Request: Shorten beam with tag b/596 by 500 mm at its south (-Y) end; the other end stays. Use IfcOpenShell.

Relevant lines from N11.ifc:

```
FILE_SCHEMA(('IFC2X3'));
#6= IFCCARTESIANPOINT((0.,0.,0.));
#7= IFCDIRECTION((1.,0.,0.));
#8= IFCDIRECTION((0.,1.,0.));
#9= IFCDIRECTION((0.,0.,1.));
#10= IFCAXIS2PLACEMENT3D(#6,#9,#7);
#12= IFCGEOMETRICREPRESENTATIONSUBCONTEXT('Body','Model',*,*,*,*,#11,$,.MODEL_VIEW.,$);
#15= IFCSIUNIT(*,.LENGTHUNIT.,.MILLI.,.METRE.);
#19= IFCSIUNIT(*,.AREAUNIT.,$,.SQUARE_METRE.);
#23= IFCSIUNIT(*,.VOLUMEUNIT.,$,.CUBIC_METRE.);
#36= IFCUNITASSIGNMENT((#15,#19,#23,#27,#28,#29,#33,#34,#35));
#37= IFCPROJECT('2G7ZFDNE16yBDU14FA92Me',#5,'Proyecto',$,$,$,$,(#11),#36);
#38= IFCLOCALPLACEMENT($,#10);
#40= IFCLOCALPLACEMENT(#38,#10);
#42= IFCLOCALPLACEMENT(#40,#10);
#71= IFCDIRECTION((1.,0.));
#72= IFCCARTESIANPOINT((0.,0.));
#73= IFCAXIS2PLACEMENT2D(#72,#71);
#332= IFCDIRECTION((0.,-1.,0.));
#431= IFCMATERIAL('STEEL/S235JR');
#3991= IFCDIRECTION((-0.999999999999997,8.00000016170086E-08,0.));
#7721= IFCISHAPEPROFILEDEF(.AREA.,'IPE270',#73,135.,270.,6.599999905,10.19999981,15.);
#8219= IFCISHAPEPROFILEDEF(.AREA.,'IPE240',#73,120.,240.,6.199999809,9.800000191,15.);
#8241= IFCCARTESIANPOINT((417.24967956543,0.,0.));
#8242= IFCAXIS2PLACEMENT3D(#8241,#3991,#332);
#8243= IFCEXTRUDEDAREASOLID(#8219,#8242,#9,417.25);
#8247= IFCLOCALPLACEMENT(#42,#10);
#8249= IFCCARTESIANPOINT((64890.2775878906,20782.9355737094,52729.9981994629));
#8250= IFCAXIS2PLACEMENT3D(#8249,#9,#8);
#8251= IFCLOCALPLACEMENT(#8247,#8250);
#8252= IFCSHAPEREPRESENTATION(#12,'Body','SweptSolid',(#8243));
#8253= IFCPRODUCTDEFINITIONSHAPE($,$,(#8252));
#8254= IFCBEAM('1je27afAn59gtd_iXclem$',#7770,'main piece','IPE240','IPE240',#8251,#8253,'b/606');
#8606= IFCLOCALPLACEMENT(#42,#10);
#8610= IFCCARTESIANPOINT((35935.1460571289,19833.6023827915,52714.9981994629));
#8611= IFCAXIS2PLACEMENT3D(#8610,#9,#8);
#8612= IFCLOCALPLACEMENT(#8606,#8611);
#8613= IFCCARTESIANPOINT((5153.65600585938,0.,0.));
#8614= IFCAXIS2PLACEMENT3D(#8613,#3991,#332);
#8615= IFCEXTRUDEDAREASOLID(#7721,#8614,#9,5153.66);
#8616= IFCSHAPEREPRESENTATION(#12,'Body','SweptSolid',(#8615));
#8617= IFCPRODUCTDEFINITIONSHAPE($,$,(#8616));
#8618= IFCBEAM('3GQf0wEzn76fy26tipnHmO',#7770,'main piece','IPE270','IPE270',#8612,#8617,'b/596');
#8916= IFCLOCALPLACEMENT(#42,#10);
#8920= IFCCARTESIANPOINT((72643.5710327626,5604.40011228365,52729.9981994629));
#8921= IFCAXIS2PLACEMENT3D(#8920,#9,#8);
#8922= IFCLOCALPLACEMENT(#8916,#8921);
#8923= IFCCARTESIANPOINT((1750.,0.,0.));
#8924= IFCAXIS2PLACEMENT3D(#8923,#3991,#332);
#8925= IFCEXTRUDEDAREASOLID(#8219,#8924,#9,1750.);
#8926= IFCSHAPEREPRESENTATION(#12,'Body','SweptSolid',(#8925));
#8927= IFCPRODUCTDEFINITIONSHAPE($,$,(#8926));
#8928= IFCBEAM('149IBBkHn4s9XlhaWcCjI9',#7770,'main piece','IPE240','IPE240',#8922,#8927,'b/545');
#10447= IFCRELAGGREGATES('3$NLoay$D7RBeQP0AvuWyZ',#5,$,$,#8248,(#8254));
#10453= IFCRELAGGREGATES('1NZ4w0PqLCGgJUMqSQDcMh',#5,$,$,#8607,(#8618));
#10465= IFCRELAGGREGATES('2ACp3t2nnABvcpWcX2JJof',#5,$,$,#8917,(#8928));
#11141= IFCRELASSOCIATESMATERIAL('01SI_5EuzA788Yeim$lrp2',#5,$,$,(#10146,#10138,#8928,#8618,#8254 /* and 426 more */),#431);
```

```python
import ifcopenshell
import ifcopenshell.util.representation

model = ifcopenshell.open("N11.ifc")

member = model.by_guid("3GQf0wEzn76fy26tipnHmO")
change = -500.0

# The extrusion runs towards the end named, so only its depth changes.
body = ifcopenshell.util.representation.get_representation(member, "Model", "Body")
solid = body.Items[0]
old_length = solid.Depth
solid.Depth += change

print(f"length {old_length:g} -> {solid.Depth:g}")

model.write("N11_v2.ifc")
```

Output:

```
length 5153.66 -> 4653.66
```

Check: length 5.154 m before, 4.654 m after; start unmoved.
